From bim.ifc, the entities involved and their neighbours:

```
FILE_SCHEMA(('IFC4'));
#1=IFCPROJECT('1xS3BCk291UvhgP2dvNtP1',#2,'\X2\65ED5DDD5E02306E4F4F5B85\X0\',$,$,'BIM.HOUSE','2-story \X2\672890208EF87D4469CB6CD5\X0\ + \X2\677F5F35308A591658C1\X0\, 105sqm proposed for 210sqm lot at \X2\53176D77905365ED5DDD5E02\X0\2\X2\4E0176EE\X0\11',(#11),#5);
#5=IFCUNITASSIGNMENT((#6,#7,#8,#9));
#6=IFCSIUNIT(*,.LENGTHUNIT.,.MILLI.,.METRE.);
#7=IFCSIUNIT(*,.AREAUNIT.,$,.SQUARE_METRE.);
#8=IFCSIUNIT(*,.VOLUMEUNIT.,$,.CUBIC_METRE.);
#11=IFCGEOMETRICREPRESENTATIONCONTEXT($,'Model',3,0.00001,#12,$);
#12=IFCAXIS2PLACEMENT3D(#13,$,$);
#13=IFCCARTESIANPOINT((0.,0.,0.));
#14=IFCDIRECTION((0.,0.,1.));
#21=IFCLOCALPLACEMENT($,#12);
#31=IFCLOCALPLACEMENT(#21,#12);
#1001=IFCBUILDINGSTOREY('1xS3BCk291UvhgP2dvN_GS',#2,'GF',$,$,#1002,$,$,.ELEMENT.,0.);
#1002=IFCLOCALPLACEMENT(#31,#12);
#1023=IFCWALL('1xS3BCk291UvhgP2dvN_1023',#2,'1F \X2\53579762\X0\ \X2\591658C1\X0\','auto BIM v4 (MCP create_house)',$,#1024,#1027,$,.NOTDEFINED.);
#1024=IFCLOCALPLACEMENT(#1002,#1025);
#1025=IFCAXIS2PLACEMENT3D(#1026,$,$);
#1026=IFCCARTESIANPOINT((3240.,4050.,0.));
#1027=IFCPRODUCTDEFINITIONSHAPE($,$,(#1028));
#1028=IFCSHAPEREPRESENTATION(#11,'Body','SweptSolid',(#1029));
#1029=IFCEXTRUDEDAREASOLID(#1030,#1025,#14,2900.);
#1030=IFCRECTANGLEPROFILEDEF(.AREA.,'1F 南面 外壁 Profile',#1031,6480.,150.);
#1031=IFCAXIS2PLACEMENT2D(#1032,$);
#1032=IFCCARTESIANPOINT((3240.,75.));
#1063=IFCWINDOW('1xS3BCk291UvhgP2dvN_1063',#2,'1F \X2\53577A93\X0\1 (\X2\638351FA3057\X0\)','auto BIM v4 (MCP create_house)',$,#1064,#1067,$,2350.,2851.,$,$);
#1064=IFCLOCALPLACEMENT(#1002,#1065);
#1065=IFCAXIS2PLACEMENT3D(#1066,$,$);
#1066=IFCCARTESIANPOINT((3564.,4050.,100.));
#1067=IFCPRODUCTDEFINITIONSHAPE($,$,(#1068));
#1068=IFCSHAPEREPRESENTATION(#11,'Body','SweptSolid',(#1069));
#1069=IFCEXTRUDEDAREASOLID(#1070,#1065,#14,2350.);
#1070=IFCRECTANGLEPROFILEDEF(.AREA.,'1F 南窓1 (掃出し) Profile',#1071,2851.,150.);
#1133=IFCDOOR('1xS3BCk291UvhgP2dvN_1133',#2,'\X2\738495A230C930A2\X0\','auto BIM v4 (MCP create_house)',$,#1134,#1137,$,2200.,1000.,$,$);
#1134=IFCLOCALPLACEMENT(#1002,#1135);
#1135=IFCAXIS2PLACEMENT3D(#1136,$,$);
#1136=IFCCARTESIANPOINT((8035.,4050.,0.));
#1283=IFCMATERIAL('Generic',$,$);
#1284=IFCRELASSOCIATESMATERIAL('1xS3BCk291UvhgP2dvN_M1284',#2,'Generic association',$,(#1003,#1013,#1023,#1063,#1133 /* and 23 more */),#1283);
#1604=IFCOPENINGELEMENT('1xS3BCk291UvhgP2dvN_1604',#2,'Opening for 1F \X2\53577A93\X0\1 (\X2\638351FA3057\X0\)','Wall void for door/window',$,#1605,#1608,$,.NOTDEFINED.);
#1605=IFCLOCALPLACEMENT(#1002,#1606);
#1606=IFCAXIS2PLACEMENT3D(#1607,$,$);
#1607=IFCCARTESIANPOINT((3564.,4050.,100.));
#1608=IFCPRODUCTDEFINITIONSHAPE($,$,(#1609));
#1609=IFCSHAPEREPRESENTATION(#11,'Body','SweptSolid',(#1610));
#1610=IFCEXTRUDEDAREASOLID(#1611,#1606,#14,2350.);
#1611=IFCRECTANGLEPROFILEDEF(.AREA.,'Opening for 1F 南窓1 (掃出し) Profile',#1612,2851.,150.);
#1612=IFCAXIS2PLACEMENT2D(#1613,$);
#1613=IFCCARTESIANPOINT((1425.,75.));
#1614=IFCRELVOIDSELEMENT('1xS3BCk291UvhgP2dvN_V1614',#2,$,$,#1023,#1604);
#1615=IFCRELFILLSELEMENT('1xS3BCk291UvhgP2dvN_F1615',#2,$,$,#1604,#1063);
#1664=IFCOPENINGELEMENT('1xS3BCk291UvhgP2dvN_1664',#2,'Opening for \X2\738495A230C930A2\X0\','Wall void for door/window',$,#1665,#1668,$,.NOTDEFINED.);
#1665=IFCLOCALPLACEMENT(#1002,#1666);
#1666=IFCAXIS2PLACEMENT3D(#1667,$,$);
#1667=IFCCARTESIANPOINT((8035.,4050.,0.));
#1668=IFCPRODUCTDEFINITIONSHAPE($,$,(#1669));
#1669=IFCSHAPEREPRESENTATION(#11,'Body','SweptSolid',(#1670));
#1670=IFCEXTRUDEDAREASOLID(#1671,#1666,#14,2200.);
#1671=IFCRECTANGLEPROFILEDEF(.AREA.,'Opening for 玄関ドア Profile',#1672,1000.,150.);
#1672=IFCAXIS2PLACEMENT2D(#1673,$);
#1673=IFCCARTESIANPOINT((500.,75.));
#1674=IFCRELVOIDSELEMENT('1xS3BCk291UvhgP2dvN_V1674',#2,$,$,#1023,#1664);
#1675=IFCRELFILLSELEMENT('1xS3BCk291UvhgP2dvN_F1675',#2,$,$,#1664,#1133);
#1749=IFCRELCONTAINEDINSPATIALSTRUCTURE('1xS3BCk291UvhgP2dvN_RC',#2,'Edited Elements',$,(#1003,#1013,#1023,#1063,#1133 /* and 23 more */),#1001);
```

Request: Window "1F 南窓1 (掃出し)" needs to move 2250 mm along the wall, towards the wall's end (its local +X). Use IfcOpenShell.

```python
import ifcopenshell
import ifcopenshell.api.geometry
import ifcopenshell.util.placement
import ifcopenshell.util.unit

model = ifcopenshell.open("bim.ifc")
unit_scale = ifcopenshell.util.unit.calculate_unit_scale(model)

window = model.by_guid("1xS3BCk291UvhgP2dvN_1063")
opening = window.FillsVoids[0].RelatingOpeningElement
wall = opening.VoidsElements[0].RelatingBuildingElement

wall_matrix = ifcopenshell.util.placement.get_local_placement(wall.ObjectPlacement)
shift = wall_matrix[:3, 0] * 2.25 / unit_scale
before = ifcopenshell.util.placement.get_local_placement(window.ObjectPlacement)[:3, 3].copy()

# The window is not placed relative to its opening, so move both.
for product in (opening, window):
    matrix = ifcopenshell.util.placement.get_local_placement(product.ObjectPlacement)
    matrix[:3, 3] += shift
    ifcopenshell.api.geometry.edit_object_placement(model, product=product, matrix=matrix, is_si=False)

after = ifcopenshell.util.placement.get_local_placement(window.ObjectPlacement)[:3, 3]
print("window moved by", (after - before).round(3) + 0.0)

model.write("bim-out.ifc")
```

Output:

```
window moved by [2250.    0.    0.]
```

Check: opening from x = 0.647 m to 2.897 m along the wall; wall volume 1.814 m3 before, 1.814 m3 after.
